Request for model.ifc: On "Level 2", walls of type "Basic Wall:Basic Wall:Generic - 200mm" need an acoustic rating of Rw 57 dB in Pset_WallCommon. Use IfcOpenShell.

First a look at what the model holds.

```python
import ifcopenshell
import ifcopenshell.util.element

model = ifcopenshell.open("model.ifc")
print(model.schema)
storey = next(s for s in model.by_type("IfcBuildingStorey") if s.Name == "Level 2")
walls = [e for e in ifcopenshell.util.element.get_decomposition(storey) if e.is_a("IfcWall")]
seen = {}
for e in walls:
    element_type = ifcopenshell.util.element.get_type(e)
    key = (element_type.Name if element_type != e and element_type else None, ifcopenshell.util.element.get_pset(e, "Pset_WallCommon", "AcousticRating"))
    seen[key] = seen.get(key, 0) + 1
for (name, value), count in sorted(seen.items(), key=str):
    print(count, "x", name, "|", value)
```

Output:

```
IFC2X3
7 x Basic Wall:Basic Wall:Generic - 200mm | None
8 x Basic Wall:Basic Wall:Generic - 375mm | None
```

```python
import ifcopenshell
import ifcopenshell.api.pset
import ifcopenshell.util.element

model = ifcopenshell.open("model.ifc")

storey = next(s for s in model.by_type("IfcBuildingStorey") if s.Name == "Level 2")
walls = [e for e in ifcopenshell.util.element.get_decomposition(storey) if e.is_a("IfcWall")]

count = 0
for e in walls:
    element_type = ifcopenshell.util.element.get_type(e)
    if element_type in (None, e) or element_type.Name != "Basic Wall:Basic Wall:Generic - 200mm":
        continue
    # add_pset returns the element's existing set when there is one.
    pset = ifcopenshell.api.pset.add_pset(model, product=e, name="Pset_WallCommon")
    ifcopenshell.api.pset.edit_pset(model, pset=pset, properties={"AcousticRating": "Rw 57 dB"})
    count += 1

print(count, "walls updated")

model.write("model_edited.ifc")
```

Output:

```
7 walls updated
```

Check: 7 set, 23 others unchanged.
